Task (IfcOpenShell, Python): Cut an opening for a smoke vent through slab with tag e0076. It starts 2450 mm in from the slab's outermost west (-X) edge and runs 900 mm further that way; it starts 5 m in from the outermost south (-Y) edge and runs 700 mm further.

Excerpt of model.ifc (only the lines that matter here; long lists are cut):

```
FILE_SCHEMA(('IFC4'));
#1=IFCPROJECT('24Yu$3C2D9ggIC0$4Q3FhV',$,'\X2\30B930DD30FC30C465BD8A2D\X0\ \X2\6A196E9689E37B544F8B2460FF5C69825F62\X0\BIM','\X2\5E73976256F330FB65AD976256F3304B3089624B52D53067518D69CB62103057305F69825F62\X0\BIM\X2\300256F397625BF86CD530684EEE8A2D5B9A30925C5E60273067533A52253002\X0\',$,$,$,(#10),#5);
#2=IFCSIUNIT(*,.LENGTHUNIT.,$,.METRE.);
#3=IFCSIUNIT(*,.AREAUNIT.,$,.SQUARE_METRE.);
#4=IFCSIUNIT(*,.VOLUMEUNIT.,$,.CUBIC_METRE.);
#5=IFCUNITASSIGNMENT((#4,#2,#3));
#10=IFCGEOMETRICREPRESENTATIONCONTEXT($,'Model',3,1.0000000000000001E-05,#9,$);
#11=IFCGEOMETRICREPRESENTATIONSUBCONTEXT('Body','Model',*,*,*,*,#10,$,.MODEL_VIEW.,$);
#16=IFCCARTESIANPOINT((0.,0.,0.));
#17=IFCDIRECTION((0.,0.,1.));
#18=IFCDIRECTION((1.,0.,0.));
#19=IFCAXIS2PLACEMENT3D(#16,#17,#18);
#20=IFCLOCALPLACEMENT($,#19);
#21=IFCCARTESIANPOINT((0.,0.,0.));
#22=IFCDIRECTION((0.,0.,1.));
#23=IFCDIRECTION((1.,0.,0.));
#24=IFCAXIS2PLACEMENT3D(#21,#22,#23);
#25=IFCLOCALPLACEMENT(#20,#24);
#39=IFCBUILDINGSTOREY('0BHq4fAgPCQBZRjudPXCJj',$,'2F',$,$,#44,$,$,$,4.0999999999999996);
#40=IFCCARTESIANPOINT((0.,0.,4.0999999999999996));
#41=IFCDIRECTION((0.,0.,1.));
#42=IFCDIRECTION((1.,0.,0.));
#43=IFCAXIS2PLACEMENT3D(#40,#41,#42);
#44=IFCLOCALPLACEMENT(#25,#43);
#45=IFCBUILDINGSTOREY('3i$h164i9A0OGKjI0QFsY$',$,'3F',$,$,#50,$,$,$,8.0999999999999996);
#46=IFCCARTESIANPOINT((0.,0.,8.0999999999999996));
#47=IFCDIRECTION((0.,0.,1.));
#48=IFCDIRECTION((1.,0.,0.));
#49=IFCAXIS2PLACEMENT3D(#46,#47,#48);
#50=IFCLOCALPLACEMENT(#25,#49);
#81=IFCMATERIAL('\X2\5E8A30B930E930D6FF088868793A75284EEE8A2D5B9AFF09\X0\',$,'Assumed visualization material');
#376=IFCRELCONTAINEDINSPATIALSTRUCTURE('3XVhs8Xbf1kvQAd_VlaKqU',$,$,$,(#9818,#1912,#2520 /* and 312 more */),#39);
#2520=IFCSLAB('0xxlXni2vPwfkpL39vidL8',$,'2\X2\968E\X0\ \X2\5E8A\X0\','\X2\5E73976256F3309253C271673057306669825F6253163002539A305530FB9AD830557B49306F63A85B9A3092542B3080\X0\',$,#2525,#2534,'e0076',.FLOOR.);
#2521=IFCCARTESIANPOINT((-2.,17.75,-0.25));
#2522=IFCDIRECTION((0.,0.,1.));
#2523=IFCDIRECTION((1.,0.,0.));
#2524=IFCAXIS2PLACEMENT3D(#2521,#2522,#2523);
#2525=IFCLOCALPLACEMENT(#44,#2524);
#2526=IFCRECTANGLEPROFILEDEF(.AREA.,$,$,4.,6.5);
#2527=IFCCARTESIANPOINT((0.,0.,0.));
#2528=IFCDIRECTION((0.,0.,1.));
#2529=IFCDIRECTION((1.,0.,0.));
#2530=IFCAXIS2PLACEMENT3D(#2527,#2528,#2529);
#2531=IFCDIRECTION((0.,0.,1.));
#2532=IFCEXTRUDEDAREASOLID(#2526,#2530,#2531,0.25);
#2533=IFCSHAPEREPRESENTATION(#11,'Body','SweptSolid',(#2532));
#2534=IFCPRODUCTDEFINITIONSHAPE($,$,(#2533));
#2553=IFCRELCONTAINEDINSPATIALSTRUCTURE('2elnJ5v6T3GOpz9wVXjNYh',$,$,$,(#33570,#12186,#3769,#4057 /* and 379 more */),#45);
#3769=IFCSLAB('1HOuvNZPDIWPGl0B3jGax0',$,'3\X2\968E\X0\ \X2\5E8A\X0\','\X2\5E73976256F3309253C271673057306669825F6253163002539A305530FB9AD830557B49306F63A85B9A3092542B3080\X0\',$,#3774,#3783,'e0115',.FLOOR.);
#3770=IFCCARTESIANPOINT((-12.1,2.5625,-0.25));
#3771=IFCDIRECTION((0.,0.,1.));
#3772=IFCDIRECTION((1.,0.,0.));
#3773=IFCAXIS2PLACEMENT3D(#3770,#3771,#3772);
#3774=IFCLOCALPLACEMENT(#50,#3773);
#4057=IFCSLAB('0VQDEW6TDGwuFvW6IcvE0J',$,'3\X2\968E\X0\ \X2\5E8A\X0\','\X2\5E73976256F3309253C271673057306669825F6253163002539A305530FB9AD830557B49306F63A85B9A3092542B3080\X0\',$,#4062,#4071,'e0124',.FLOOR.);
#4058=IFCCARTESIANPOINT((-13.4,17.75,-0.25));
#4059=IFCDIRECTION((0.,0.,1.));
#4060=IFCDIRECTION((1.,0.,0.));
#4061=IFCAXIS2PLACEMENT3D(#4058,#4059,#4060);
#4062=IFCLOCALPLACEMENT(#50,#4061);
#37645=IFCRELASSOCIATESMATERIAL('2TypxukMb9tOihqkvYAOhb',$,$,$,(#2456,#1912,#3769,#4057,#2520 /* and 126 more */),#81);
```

```python
import numpy as np
import ifcopenshell
import ifcopenshell.api.feature
import ifcopenshell.api.geometry
import ifcopenshell.api.root
import ifcopenshell.geom
import ifcopenshell.util.placement
import ifcopenshell.util.representation
import ifcopenshell.util.shape
import ifcopenshell.util.unit

model = ifcopenshell.open("model.ifc")
unit_scale = ifcopenshell.util.unit.calculate_unit_scale(model)
settings = ifcopenshell.geom.settings()


def volume(element):
    """Net volume in cubic metres, openings subtracted."""
    shape = ifcopenshell.geom.create_shape(settings, element)
    return ifcopenshell.util.shape.get_volume(shape.geometry)


slab = model.by_guid("0xxlXni2vPwfkpL39vidL8")
before = volume(slab)

# Extent in the slab's own axes, in metres. The edges named are its -X and -Y sides.
slab_shape = ifcopenshell.geom.create_shape(settings, slab)
vertices = ifcopenshell.util.shape.get_vertices(slab_shape.geometry)
x_min, y_min, bottom = vertices.min(axis=0)
top = vertices[:, 2].max()

opening = ifcopenshell.api.root.create_entity(model, ifc_class="IfcOpeningElement", name="Smoke vent opening", predefined_type="OPENING")
context = ifcopenshell.util.representation.get_context(model, "Model", "Body", "MODEL_VIEW")
width, depth = 0.9, 0.7
outline = [(0.0, 0.0), (width, 0.0), (width, depth), (0.0, depth), (0.0, 0.0)]
# Overshoot both faces by 50 mm so the cut is clean.
shape = ifcopenshell.api.geometry.add_slab_representation(
    model, context=context, depth=top - bottom + 0.1, polyline=outline
)
ifcopenshell.api.geometry.assign_representation(model, product=opening, representation=shape)

matrix = ifcopenshell.util.placement.get_local_placement(slab.ObjectPlacement)
matrix[:, 3] = matrix @ np.append(np.array([x_min + 2.45, y_min + 5, bottom - 0.05]) / unit_scale, 1.0)
ifcopenshell.api.geometry.edit_object_placement(model, product=opening, matrix=matrix, is_si=False)
ifcopenshell.api.feature.add_feature(model, feature=opening, element=slab)

after = volume(slab)

print(f"slab volume {before:.3f} -> {after:.3f} m3")

model.write("model_rev.ifc")
```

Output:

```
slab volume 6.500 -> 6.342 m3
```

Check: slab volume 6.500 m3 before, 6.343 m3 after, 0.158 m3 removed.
